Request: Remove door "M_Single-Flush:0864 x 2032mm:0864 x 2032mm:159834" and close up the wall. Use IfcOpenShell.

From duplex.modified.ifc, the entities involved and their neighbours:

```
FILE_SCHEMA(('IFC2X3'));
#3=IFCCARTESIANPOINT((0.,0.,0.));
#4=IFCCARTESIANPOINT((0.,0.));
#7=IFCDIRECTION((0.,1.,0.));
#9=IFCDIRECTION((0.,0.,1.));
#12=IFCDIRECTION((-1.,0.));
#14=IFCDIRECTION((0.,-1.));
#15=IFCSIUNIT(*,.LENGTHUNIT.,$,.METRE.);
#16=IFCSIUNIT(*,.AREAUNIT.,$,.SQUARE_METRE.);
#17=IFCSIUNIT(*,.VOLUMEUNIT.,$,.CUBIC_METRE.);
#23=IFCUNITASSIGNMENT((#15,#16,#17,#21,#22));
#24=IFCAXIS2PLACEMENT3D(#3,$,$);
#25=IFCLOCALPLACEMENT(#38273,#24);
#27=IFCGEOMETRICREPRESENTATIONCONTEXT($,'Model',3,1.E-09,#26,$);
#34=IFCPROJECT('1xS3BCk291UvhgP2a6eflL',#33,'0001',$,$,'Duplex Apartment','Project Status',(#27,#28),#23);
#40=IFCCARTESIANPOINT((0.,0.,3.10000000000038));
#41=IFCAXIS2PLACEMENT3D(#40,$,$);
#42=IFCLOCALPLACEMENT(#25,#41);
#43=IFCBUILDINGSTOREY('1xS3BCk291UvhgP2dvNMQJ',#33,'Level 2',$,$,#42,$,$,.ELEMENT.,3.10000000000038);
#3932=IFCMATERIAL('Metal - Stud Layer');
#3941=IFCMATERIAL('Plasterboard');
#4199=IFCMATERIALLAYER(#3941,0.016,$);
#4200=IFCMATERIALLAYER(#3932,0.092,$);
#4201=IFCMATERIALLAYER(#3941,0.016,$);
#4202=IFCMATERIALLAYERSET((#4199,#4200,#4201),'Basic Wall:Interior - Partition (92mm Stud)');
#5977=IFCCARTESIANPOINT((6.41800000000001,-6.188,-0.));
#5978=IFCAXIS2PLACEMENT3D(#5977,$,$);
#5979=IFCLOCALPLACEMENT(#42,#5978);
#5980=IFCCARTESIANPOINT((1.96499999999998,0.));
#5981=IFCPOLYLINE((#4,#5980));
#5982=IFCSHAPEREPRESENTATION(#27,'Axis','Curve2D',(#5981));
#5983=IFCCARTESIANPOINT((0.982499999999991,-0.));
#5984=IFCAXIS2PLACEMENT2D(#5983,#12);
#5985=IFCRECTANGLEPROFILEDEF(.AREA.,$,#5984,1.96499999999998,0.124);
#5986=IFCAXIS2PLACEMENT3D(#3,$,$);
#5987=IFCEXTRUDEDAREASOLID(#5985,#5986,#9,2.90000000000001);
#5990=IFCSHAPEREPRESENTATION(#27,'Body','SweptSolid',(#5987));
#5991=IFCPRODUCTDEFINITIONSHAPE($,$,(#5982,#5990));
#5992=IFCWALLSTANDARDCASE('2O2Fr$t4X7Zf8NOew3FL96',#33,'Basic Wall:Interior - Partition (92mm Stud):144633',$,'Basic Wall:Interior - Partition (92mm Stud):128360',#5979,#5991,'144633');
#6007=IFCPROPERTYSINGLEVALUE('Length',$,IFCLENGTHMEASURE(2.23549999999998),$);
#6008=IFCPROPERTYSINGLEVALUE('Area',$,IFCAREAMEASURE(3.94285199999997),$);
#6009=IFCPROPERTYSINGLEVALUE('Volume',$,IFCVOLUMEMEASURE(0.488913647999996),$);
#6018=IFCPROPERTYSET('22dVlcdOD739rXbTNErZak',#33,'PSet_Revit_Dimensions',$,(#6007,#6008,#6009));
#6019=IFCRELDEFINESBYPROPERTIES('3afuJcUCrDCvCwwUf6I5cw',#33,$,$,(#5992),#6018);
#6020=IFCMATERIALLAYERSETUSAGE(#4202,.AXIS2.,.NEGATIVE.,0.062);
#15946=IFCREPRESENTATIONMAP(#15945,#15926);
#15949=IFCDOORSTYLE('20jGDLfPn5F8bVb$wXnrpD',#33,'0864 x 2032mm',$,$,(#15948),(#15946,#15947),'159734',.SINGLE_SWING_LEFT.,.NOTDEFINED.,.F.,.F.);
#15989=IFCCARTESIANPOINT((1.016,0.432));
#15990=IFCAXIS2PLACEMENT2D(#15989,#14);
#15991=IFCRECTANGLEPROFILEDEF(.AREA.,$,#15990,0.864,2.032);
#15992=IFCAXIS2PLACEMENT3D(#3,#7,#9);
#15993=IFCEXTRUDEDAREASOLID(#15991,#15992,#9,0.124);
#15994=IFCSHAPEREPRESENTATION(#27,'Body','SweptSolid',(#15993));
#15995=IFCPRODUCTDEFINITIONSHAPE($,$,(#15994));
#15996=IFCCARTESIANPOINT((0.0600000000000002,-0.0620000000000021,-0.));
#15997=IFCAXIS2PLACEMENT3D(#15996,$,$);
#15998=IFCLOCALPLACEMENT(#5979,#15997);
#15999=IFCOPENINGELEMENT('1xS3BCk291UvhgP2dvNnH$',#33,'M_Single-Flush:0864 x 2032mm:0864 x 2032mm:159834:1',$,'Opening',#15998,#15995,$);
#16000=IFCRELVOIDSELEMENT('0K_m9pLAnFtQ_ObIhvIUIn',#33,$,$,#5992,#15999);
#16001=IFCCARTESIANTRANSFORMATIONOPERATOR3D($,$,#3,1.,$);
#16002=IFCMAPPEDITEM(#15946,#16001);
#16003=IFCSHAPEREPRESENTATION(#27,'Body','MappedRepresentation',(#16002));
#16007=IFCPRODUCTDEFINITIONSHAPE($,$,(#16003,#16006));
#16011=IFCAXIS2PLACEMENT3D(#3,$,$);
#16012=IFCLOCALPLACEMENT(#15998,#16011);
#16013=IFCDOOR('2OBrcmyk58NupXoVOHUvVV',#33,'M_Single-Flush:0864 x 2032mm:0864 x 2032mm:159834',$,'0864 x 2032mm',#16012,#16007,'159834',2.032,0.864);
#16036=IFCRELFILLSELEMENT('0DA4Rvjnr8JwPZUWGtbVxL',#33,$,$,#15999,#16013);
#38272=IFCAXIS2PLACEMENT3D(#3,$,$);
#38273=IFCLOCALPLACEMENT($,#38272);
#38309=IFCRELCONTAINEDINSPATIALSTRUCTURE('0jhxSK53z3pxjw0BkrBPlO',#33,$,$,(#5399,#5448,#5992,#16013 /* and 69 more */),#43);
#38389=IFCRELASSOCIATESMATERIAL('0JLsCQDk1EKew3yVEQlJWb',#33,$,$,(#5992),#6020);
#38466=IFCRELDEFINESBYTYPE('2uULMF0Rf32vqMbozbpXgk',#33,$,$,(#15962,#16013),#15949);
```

```python
import ifcopenshell
import ifcopenshell.api.feature
import ifcopenshell.api.pset
import ifcopenshell.api.root
import ifcopenshell.geom
import ifcopenshell.util.element
import ifcopenshell.util.shape
import ifcopenshell.util.unit

model = ifcopenshell.open("duplex.modified.ifc")
area_scale = ifcopenshell.util.unit.calculate_unit_scale(model, "AREAUNIT")
volume_scale = ifcopenshell.util.unit.calculate_unit_scale(model, "VOLUMEUNIT")
settings = ifcopenshell.geom.settings()


def volume(element):
    """Net volume in cubic metres, openings subtracted."""
    shape = ifcopenshell.geom.create_shape(settings, element)
    return ifcopenshell.util.shape.get_volume(shape.geometry)


door = model.by_guid("2OBrcmyk58NupXoVOHUvVV")
opening = door.FillsVoids[0].RelatingOpeningElement
wall = opening.VoidsElements[0].RelatingBuildingElement
before = volume(wall)

ifcopenshell.api.root.remove_product(model, product=door)
ifcopenshell.api.feature.remove_feature(model, feature=opening)

after = volume(wall)
thickness = 0.124  # wall thickness in metres

# Update the wall's stored quantities.
pset = model.by_id(ifcopenshell.util.element.get_pset(wall, "PSet_Revit_Dimensions", should_inherit=False)["id"])
ifcopenshell.api.pset.edit_pset(model, pset=pset, properties={
    "Area": model.create_entity("IfcAreaMeasure", after / thickness / area_scale),
    "Volume": model.create_entity("IfcVolumeMeasure", after / volume_scale),
})

print(f"wall volume {before:.3f} -> {after:.3f} m3")

model.write("duplex.modified_edited.ifc")
```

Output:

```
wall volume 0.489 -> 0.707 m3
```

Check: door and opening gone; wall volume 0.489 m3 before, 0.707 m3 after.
